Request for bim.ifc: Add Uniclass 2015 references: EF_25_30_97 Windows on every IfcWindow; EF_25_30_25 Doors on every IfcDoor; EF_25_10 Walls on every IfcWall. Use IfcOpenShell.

First a look at what the model holds.

```python
import ifcopenshell

model = ifcopenshell.open("bim.ifc")
print(model.schema)
print("classifications:", [c.Name for c in model.by_type("IfcClassification")])
for ifc_class in ("IfcDoor", "IfcRoof", "IfcStair", "IfcWall", "IfcWindow"):
    print(ifc_class, len(model.by_type(ifc_class)))
```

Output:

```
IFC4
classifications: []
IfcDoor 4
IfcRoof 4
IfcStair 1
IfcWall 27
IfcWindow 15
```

```python
import ifcopenshell
import ifcopenshell.api.classification

model = ifcopenshell.open("bim.ifc")

system = ifcopenshell.api.classification.add_classification(model, classification="Uniclass 2015")

codes = {
    "IfcWindow": ("EF_25_30_97", "Windows"),
    "IfcDoor": ("EF_25_30_25", "Doors"),
    "IfcWall": ("EF_25_10", "Walls"),
}
for ifc_class, (code, name) in codes.items():
    products = model.by_type(ifc_class)
    ifcopenshell.api.classification.add_reference(
        model, products=products, classification=system, identification=code, name=name
    )
    print(code, len(products))

model.write("bim_rev.ifc")
```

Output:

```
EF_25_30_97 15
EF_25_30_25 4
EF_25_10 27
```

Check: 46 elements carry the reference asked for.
